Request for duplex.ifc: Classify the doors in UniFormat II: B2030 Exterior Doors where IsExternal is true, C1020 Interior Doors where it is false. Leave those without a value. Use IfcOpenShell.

First a look at what the model holds.

```python
import ifcopenshell
import ifcopenshell.util.element

model = ifcopenshell.open("duplex.ifc")
print(model.schema)
print("classifications:", [c.Name for c in model.by_type("IfcClassification")])
values = [ifcopenshell.util.element.get_pset(e, "Pset_DoorCommon", "IsExternal") for e in model.by_type("IfcDoor")]
for value in (True, False, None):
    print("IsExternal", value, values.count(value))
```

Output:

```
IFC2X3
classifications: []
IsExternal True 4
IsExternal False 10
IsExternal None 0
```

```python
import ifcopenshell
import ifcopenshell.api.classification
import ifcopenshell.util.element

model = ifcopenshell.open("duplex.ifc")

# IFC2X3 requires Source and Edition and has no link from the project to the system.
system = model.create_entity("IfcClassification", Source="ASTM", Edition="E1557", Name="UniFormat II")

doors = model.by_type("IfcDoor")
external = {e: ifcopenshell.util.element.get_pset(e, "Pset_DoorCommon", "IsExternal") for e in doors}
for flag, code, name in ((True, "B2030", "Exterior Doors"), (False, "C1020", "Interior Doors")):
    products = [e for e in doors if external[e] is flag]
    ifcopenshell.api.classification.add_reference(
        model, products=products, classification=system, identification=code, name=name
    )
    print(code, len(products))

model.write("duplex-out.ifc")
```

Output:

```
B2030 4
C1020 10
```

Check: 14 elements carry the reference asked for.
